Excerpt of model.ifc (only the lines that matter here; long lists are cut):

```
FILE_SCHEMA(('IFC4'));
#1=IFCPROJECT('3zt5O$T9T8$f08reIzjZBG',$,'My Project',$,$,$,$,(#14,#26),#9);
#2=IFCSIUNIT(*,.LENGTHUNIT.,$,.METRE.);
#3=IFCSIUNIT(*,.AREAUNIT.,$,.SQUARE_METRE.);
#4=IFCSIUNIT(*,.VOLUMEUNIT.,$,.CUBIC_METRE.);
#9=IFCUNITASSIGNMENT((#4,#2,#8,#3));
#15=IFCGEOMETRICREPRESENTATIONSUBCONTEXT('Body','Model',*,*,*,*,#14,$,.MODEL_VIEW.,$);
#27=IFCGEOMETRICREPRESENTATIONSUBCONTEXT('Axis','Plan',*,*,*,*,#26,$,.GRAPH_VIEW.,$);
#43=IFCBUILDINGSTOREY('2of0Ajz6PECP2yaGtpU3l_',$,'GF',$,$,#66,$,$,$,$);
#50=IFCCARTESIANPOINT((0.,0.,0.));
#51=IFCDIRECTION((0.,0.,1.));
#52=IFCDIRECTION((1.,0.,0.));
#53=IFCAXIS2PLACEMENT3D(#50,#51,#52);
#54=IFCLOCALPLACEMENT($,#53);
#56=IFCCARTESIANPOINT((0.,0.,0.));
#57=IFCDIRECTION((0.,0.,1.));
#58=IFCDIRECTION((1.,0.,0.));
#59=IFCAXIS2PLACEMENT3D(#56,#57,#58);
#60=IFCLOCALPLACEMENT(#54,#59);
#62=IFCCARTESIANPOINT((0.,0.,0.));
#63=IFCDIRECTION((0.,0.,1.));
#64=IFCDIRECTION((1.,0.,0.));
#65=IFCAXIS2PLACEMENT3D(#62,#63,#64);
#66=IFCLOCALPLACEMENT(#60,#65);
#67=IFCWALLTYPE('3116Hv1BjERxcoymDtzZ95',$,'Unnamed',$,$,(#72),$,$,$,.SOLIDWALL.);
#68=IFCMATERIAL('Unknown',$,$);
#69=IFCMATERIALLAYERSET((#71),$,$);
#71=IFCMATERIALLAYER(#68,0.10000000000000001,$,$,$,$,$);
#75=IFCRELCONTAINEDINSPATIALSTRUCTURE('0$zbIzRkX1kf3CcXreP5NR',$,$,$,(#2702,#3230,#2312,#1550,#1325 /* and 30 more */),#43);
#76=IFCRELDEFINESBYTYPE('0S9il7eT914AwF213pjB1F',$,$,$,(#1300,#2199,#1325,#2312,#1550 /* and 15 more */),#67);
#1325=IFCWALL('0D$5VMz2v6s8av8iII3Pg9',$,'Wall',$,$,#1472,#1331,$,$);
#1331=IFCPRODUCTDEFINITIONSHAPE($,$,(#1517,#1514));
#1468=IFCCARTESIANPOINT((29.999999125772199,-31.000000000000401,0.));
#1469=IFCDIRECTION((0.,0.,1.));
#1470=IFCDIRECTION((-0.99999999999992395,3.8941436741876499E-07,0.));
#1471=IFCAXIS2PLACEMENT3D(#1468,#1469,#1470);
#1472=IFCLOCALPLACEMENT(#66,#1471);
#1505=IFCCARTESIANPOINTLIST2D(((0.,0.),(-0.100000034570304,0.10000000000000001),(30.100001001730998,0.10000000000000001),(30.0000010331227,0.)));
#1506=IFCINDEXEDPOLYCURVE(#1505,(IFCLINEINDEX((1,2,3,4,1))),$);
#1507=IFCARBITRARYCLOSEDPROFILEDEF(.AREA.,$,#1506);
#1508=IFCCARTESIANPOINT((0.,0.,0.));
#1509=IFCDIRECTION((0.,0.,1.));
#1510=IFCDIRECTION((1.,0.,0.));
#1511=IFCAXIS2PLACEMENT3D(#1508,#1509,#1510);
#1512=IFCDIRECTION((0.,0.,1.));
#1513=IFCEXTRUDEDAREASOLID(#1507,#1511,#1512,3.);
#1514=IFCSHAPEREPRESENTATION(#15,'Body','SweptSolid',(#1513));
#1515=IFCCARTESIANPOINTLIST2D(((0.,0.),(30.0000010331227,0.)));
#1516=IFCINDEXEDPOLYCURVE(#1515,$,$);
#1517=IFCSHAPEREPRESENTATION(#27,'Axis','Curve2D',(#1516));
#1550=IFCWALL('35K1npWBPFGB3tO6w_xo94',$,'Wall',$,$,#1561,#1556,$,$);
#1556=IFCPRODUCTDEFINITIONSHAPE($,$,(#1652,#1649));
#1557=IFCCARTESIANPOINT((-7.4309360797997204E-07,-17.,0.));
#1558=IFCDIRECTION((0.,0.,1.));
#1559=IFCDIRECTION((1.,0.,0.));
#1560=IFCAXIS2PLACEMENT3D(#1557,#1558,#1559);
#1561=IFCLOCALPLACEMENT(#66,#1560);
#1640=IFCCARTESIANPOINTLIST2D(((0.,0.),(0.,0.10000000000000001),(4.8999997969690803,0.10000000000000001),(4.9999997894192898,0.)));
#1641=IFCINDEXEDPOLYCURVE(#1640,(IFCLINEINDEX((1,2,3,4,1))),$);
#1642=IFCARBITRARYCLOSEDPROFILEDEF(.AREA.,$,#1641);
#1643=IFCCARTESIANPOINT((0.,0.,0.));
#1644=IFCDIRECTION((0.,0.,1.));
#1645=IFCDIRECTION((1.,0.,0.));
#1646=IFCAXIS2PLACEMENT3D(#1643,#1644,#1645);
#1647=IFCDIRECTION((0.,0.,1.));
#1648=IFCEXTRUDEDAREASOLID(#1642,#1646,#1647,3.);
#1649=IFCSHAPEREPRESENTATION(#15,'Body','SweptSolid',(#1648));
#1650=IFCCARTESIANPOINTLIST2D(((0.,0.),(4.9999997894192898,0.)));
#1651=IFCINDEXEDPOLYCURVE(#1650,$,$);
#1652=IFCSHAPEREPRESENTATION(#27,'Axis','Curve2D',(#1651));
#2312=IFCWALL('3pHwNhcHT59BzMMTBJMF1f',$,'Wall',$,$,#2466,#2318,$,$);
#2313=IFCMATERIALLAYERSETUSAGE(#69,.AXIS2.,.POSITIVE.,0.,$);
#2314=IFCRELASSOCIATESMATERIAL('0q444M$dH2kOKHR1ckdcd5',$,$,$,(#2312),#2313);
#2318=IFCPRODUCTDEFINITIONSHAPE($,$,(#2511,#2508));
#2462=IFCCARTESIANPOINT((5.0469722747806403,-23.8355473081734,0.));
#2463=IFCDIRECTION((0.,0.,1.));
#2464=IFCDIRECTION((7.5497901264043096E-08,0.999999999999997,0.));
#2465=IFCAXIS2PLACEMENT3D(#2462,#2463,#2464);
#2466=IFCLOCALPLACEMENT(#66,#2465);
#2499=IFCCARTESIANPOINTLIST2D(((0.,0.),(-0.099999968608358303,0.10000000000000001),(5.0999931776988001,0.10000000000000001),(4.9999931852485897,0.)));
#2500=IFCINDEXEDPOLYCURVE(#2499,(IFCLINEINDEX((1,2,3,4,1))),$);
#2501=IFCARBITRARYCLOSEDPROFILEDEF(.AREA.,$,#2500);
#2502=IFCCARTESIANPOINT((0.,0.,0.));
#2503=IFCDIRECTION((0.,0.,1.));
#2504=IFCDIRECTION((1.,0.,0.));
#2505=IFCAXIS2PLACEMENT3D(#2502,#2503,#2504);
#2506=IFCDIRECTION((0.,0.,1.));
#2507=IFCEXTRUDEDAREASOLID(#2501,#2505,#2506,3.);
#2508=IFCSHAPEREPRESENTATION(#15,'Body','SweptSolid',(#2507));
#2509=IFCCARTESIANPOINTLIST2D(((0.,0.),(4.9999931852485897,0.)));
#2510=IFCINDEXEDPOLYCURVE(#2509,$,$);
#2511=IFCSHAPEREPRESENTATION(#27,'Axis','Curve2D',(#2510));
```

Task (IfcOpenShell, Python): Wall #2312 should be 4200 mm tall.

```python
import ifcopenshell
import ifcopenshell.geom
import ifcopenshell.util.representation
import ifcopenshell.util.shape
import ifcopenshell.util.unit

model = ifcopenshell.open("model.ifc")
unit_scale = ifcopenshell.util.unit.calculate_unit_scale(model)
settings = ifcopenshell.geom.settings()


def volume(element):
    """Net volume in cubic metres, openings subtracted."""
    shape = ifcopenshell.geom.create_shape(settings, element)
    return ifcopenshell.util.shape.get_volume(shape.geometry)


wall = model.by_guid("3pHwNhcHT59BzMMTBJMF1f")
before = volume(wall)

body = ifcopenshell.util.representation.get_representation(wall, "Model", "Body")
solid = body.Items[0]
old_height = solid.Depth
solid.Depth = 4.2 / unit_scale
after = volume(wall)

print(f"height {old_height:g} -> {solid.Depth:g}, volume {before:.3f} -> {after:.3f} m3")

model.write("model_updated.ifc")
```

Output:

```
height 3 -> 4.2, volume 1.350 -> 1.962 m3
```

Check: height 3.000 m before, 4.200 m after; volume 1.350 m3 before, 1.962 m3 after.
